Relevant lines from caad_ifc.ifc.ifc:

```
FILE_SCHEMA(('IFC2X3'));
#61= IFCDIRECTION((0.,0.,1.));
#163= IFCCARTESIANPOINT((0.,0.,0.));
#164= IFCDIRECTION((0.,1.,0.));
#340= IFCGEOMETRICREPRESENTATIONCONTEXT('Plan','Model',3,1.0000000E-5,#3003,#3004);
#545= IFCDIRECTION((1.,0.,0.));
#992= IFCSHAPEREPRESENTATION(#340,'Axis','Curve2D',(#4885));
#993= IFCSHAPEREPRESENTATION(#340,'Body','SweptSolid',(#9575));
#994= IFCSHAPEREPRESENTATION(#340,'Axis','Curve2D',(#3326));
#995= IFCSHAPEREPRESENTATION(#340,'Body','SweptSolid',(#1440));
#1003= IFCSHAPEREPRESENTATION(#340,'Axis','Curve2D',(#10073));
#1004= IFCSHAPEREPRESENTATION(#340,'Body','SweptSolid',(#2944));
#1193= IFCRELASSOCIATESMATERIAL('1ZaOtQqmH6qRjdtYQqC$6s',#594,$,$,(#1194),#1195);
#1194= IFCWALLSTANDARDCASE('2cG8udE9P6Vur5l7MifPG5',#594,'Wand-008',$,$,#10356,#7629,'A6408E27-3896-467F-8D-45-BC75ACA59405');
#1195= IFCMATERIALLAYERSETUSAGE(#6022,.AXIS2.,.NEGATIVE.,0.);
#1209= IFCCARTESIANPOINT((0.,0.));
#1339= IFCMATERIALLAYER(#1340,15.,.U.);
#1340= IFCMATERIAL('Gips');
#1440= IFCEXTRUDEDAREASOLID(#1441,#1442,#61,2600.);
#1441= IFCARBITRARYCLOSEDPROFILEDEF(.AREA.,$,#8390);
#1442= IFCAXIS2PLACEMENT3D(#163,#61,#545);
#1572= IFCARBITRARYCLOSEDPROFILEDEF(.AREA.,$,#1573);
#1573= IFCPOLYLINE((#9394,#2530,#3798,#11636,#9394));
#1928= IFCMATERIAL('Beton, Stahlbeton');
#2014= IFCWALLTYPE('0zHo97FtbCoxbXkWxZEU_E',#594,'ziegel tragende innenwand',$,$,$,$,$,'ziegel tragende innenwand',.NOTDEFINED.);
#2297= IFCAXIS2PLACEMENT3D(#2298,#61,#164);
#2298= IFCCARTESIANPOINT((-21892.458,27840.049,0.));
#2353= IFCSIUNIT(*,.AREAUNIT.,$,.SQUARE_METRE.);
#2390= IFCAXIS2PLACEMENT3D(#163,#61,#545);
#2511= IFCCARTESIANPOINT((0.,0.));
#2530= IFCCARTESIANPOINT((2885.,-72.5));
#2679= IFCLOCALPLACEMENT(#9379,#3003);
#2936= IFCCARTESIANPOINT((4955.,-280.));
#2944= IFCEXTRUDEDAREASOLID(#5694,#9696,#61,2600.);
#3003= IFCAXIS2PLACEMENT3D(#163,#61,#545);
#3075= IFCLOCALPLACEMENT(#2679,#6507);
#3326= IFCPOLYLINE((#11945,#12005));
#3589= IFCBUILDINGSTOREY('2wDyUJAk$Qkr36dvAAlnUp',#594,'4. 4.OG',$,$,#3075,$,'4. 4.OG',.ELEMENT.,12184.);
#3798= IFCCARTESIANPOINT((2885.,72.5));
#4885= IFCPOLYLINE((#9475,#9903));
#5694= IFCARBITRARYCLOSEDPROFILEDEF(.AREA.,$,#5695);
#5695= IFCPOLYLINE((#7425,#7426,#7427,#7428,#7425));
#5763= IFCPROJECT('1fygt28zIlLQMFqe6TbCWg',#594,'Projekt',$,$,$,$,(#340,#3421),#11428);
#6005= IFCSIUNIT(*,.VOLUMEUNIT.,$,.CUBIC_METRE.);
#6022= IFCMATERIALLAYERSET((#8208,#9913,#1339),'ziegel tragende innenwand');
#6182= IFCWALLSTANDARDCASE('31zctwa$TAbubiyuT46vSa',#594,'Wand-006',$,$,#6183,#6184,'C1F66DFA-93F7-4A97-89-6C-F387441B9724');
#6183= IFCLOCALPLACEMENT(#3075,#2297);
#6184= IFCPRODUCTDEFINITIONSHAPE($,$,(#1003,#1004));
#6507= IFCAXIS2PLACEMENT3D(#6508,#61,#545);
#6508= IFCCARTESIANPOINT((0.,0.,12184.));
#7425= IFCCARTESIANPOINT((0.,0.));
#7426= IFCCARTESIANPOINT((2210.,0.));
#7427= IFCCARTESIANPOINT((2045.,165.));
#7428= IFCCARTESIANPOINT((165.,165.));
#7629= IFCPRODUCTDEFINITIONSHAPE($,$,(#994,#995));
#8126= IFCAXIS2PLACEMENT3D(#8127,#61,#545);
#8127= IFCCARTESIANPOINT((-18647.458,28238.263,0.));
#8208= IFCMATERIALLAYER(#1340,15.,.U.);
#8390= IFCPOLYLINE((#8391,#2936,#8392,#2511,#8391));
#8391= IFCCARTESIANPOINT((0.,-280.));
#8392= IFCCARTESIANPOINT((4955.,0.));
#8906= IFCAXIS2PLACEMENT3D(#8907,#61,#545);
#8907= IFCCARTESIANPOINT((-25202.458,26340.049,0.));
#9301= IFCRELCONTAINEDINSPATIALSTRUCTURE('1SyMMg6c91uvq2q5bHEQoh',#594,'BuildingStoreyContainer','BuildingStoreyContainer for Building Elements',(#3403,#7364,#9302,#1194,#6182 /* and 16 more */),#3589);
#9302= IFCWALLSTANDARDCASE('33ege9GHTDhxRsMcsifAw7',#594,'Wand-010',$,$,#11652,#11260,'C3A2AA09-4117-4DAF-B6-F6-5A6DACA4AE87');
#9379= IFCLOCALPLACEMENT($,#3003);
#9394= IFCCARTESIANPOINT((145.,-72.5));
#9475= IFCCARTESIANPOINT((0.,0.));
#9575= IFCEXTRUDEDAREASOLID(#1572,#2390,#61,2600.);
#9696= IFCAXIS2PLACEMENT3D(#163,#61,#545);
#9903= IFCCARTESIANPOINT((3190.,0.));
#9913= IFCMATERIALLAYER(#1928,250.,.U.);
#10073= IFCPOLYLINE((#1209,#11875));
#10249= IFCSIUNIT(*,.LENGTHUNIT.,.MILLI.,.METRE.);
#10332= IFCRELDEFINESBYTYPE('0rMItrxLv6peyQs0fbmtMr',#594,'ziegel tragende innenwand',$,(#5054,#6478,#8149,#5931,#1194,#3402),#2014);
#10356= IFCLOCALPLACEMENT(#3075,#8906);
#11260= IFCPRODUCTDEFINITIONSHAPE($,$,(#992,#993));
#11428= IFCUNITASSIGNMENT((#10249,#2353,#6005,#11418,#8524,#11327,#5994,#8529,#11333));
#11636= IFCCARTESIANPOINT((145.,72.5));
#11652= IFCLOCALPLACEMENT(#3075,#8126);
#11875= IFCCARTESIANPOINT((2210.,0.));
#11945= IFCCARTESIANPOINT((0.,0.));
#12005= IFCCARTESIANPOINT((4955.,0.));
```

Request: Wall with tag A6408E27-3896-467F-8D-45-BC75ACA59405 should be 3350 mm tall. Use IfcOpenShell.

```python
import ifcopenshell
import ifcopenshell.geom
import ifcopenshell.util.shape

model = ifcopenshell.open("caad_ifc.ifc.ifc")
settings = ifcopenshell.geom.settings()


def volume(element):
    """Net volume in cubic metres, openings subtracted."""
    shape = ifcopenshell.geom.create_shape(settings, element)
    return ifcopenshell.util.shape.get_volume(shape.geometry)


wall = model.by_id(1194)
before = volume(wall)

body = next(r for r in wall.Representation.Representations if r.RepresentationIdentifier == "Body")
solid = body.Items[0]
old_height = solid.Depth
solid.Depth = 3350.0
after = volume(wall)

print(f"height {old_height:g} -> {solid.Depth:g}, volume {before:.3f} -> {after:.3f} m3")

model.write("caad_ifc.ifc-out.ifc")
```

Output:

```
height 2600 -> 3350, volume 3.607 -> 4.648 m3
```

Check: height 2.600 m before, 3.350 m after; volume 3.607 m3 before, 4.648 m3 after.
